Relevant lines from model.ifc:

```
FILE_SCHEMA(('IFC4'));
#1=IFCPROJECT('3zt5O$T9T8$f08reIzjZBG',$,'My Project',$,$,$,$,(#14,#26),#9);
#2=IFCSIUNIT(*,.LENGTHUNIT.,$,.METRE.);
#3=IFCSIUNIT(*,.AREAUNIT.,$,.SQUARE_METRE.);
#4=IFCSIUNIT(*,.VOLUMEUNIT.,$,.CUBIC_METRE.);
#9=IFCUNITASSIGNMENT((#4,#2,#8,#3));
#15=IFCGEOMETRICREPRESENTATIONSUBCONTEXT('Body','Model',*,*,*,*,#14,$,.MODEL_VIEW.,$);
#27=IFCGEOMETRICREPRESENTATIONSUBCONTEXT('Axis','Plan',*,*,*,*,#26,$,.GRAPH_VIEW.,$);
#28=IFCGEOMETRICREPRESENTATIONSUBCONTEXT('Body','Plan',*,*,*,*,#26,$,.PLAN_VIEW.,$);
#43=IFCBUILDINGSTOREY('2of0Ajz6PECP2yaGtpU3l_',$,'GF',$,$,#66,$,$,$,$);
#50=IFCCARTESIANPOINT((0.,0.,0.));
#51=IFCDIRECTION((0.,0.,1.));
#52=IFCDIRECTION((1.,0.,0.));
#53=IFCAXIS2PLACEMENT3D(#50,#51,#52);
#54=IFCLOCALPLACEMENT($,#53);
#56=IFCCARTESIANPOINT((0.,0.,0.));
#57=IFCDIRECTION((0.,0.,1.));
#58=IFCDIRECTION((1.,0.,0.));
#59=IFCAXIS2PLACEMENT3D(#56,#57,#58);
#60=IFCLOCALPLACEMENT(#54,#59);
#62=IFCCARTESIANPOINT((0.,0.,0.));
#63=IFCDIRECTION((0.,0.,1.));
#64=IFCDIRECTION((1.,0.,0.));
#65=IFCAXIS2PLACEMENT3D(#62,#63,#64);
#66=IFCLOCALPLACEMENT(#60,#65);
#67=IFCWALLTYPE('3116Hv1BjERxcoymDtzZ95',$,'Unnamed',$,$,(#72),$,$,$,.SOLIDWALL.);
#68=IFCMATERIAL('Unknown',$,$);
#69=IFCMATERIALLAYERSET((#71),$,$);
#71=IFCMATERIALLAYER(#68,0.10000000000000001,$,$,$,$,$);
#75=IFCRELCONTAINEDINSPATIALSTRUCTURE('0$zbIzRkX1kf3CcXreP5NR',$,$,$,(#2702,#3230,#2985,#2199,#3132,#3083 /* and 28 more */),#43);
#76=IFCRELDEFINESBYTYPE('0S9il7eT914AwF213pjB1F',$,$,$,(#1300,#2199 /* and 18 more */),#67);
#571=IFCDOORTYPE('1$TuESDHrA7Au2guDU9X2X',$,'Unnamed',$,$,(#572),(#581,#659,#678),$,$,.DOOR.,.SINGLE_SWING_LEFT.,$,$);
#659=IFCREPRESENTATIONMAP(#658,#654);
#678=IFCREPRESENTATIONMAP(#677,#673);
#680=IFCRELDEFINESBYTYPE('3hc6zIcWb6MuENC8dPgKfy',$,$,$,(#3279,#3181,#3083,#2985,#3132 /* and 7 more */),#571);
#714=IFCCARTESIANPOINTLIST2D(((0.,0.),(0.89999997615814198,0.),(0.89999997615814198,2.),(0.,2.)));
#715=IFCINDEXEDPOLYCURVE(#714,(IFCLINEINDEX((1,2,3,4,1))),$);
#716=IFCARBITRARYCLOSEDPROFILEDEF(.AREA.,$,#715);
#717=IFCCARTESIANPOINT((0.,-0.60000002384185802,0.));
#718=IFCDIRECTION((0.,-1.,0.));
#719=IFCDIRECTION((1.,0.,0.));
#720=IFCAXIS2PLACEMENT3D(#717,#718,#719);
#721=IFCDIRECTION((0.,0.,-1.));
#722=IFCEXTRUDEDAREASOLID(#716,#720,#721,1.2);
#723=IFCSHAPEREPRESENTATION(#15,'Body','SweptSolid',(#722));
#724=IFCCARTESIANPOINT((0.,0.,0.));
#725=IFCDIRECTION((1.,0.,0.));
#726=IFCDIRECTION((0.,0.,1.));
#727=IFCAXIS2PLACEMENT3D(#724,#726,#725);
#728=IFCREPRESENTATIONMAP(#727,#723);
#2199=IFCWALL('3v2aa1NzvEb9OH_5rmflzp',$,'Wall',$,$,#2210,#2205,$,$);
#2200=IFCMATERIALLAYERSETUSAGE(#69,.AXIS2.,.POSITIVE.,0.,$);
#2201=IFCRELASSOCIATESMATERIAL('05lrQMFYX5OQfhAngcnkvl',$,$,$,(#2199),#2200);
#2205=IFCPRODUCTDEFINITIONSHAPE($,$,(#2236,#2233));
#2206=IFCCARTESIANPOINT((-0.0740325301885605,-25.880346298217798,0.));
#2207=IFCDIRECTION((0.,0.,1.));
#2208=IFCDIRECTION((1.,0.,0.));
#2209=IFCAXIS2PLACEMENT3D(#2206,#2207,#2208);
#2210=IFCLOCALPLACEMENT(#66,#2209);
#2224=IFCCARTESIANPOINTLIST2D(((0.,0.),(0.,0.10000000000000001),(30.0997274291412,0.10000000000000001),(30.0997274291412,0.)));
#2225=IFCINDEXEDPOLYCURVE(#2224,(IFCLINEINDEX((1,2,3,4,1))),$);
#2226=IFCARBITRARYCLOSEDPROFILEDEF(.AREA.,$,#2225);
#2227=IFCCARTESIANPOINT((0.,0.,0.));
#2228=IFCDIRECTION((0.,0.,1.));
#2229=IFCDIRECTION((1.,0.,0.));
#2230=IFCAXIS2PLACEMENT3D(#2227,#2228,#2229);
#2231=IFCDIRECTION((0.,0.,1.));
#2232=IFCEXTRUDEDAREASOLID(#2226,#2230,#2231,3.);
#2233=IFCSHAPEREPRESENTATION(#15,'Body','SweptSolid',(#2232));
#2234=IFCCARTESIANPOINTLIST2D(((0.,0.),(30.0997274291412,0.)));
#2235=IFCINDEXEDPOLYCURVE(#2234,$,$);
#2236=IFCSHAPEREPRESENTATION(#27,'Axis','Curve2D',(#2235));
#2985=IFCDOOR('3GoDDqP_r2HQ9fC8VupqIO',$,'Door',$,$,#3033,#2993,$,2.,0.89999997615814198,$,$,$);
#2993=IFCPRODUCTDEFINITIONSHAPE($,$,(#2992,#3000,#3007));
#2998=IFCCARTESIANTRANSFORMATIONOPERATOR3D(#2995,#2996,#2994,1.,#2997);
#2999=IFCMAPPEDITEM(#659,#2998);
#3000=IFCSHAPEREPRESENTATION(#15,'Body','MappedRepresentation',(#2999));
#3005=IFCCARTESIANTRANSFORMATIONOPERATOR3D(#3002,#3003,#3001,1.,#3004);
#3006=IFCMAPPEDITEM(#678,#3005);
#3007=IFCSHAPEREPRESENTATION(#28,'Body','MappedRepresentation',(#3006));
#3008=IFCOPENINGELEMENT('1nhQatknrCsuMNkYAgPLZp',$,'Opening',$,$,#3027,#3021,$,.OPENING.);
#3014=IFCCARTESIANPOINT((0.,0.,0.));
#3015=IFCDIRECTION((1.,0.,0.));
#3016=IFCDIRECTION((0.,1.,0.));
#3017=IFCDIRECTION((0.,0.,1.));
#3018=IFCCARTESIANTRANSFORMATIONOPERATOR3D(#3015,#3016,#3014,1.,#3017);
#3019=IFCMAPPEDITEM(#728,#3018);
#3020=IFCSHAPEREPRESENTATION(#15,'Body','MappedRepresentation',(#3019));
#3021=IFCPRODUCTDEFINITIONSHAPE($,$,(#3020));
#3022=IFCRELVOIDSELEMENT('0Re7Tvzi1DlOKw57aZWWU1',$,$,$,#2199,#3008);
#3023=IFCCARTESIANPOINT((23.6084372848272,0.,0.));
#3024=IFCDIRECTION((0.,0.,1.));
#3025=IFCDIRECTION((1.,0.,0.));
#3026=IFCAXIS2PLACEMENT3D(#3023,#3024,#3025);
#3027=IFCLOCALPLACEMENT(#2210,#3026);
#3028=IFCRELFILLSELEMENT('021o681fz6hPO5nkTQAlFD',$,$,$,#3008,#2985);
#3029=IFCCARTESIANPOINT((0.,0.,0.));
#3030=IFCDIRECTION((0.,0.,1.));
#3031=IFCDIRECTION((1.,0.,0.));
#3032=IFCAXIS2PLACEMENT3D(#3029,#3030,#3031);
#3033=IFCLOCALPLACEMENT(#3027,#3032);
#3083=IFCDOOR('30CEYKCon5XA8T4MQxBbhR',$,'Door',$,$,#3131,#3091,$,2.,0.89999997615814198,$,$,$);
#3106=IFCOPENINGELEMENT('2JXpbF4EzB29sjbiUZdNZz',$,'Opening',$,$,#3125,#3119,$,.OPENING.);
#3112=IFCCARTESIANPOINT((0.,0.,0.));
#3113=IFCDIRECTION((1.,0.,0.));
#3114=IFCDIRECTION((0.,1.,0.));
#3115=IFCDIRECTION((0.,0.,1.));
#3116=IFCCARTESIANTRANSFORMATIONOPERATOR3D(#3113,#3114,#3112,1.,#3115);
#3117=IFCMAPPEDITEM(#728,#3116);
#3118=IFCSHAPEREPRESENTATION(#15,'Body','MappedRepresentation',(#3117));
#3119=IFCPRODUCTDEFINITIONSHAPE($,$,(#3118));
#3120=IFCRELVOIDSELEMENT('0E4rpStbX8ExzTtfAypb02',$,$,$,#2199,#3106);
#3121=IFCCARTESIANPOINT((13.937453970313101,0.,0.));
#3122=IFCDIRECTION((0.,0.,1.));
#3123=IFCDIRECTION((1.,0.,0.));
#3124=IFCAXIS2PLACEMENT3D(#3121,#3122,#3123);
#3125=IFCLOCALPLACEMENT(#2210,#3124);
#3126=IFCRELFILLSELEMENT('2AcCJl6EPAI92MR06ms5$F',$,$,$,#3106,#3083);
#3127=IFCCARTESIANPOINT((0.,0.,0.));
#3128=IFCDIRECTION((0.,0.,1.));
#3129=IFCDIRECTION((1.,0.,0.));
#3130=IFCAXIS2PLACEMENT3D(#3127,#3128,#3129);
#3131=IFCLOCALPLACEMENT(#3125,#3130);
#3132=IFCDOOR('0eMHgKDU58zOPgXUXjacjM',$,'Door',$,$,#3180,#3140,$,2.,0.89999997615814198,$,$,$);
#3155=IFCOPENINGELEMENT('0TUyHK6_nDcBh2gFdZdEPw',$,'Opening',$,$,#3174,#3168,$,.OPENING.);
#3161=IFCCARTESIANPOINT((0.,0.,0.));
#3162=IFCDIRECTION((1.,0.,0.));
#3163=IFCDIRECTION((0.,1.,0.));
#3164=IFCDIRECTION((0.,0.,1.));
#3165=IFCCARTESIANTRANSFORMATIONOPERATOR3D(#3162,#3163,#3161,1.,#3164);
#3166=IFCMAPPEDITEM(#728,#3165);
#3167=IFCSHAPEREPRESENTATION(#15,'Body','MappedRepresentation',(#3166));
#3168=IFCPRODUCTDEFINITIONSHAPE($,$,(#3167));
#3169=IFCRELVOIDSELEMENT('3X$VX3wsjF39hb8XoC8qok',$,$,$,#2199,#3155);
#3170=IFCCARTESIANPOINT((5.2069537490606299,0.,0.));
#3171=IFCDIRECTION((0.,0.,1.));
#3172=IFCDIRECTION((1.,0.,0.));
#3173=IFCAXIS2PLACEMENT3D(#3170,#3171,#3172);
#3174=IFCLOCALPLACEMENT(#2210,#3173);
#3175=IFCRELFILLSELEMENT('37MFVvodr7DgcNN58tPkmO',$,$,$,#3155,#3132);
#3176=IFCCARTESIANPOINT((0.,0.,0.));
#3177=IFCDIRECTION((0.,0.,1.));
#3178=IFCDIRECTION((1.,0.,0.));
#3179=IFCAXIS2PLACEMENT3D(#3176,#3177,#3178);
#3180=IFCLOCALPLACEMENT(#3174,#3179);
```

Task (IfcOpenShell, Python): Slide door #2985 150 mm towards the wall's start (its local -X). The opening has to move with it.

```python
import ifcopenshell
import ifcopenshell.api.geometry
import ifcopenshell.util.placement
import ifcopenshell.util.unit

model = ifcopenshell.open("model.ifc")
unit_scale = ifcopenshell.util.unit.calculate_unit_scale(model)

door = model.by_guid("3GoDDqP_r2HQ9fC8VupqIO")
opening = door.FillsVoids[0].RelatingOpeningElement
wall = opening.VoidsElements[0].RelatingBuildingElement

wall_matrix = ifcopenshell.util.placement.get_local_placement(wall.ObjectPlacement)
shift = wall_matrix[:3, 0] * -0.15 / unit_scale
before = ifcopenshell.util.placement.get_local_placement(door.ObjectPlacement)[:3, 3].copy()

# The door is placed relative to its opening, so it follows when the opening moves.
matrix = ifcopenshell.util.placement.get_local_placement(opening.ObjectPlacement)
matrix[:3, 3] += shift
ifcopenshell.api.geometry.edit_object_placement(
    model, product=opening, matrix=matrix, is_si=False, should_transform_children=True
)

after = ifcopenshell.util.placement.get_local_placement(door.ObjectPlacement)[:3, 3]
print("door moved by", (after - before).round(3) + 0.0)

model.write("model_edited.ifc")
```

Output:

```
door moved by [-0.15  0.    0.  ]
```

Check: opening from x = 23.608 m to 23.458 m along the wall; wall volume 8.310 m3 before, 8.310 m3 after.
